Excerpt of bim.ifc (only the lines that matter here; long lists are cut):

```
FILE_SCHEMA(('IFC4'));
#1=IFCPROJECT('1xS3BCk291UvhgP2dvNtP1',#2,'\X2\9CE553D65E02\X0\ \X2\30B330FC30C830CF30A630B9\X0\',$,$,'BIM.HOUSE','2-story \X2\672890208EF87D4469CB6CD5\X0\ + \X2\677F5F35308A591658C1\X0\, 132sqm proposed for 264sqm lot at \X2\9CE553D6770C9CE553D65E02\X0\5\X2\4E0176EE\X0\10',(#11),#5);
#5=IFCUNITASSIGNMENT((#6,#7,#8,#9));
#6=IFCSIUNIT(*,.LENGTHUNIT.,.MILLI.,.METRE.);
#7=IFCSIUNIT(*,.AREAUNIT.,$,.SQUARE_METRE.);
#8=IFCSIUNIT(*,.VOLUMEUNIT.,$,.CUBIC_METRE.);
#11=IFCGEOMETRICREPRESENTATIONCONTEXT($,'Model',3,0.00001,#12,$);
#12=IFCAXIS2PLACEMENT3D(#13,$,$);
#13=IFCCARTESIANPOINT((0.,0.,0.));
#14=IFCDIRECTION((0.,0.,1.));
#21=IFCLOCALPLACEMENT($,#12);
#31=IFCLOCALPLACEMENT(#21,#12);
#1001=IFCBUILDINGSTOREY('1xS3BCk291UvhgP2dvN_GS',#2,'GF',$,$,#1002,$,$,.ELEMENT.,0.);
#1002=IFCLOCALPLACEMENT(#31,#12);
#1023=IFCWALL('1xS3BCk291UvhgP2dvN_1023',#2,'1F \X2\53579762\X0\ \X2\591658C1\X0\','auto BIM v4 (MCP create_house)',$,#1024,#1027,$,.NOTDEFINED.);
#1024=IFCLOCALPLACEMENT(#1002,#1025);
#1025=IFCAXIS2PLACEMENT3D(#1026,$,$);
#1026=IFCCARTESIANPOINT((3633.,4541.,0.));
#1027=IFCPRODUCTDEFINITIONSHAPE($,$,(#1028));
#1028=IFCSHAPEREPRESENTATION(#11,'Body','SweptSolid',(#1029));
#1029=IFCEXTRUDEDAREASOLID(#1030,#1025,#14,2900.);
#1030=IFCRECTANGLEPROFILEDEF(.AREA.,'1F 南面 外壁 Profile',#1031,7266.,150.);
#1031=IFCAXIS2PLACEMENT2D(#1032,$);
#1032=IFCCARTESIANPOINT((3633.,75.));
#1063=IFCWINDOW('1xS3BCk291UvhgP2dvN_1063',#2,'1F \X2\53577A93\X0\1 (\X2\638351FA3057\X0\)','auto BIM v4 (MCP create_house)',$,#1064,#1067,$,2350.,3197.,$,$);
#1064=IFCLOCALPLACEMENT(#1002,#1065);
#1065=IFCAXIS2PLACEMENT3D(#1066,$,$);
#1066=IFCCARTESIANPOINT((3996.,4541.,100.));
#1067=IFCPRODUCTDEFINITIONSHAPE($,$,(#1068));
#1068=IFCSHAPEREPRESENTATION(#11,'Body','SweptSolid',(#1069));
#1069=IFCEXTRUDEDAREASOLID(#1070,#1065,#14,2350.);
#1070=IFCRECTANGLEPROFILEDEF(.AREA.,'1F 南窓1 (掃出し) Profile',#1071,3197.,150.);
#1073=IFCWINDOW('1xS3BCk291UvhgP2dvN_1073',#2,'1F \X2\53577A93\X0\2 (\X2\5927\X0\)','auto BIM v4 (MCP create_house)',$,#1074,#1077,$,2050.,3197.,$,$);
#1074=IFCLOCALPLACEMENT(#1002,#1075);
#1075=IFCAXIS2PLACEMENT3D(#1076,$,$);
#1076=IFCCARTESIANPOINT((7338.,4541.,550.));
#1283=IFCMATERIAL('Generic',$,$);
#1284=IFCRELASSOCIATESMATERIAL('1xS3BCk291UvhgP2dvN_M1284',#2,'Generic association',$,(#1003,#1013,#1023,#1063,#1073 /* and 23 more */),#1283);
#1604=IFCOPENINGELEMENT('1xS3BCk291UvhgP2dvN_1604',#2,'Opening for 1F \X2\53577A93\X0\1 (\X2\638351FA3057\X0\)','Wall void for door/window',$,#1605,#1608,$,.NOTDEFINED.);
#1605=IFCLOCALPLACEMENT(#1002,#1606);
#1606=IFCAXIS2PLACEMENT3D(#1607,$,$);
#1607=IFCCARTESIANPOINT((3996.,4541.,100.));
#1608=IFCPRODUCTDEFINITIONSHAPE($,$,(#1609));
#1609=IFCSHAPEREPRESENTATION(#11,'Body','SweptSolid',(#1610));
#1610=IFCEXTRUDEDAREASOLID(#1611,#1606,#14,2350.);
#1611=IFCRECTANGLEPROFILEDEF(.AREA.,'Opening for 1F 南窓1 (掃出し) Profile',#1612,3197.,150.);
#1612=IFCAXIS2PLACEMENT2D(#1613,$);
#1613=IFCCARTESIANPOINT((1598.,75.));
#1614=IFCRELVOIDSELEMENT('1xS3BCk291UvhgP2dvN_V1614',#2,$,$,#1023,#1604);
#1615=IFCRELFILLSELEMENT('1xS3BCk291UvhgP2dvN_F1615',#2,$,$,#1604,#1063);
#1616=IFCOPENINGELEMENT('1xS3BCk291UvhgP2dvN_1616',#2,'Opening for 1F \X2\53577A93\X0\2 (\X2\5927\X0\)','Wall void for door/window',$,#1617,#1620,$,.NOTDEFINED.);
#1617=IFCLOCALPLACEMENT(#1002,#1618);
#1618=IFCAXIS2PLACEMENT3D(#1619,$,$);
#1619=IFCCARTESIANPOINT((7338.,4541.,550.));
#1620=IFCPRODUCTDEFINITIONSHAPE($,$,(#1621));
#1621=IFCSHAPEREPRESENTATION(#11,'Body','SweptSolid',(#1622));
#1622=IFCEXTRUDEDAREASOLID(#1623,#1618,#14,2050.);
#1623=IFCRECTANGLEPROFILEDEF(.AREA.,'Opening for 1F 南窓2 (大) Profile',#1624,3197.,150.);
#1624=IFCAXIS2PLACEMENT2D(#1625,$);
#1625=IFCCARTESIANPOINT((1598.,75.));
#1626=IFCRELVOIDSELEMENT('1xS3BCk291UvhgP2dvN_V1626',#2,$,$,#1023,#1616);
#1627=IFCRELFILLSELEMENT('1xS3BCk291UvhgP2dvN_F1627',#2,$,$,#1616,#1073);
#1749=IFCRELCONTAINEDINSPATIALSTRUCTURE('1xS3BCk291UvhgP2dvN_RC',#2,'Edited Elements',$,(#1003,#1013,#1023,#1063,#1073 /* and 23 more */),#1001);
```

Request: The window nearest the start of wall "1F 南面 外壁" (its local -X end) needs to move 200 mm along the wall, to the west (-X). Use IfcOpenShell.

```python
import ifcopenshell
import ifcopenshell.api.geometry
import ifcopenshell.util.placement
import ifcopenshell.util.unit

model = ifcopenshell.open("bim.ifc")
unit_scale = ifcopenshell.util.unit.calculate_unit_scale(model)

window = model.by_id(1063)
opening = window.FillsVoids[0].RelatingOpeningElement
wall = opening.VoidsElements[0].RelatingBuildingElement

wall_matrix = ifcopenshell.util.placement.get_local_placement(wall.ObjectPlacement)
shift = wall_matrix[:3, 0] * -0.2 / unit_scale
before = ifcopenshell.util.placement.get_local_placement(window.ObjectPlacement)[:3, 3].copy()

# The window is not placed relative to its opening, so move both.
for product in (opening, window):
    matrix = ifcopenshell.util.placement.get_local_placement(product.ObjectPlacement)
    matrix[:3, 3] += shift
    ifcopenshell.api.geometry.edit_object_placement(model, product=product, matrix=matrix, is_si=False)

after = ifcopenshell.util.placement.get_local_placement(window.ObjectPlacement)[:3, 3]
print("window moved by", (after - before).round(3) + 0.0)

model.write("bim_rev.ifc")
```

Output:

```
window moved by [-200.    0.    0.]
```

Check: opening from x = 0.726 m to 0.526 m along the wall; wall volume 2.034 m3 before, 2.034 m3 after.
